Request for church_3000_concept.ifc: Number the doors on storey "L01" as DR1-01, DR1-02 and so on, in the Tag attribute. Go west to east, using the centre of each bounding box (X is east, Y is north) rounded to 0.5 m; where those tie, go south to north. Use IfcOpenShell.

First a look at what the model holds.

```python
import ifcopenshell
import ifcopenshell.util.element
import ifcopenshell.util.placement

model = ifcopenshell.open("church_3000_concept.ifc")
print(model.schema)
storey = next(s for s in model.by_type("IfcBuildingStorey") if s.Name == "L01")
doors = [e for e in ifcopenshell.util.element.get_decomposition(storey) if e.is_a("IfcDoor")]
for e in sorted(doors, key=lambda e: e.id()):
    origin = ifcopenshell.util.placement.get_local_placement(e.ObjectPlacement)[:3, 3]
    print(e.id(), e.Tag, e.Name, origin.round(2) + 0.0, sep=" | ")
```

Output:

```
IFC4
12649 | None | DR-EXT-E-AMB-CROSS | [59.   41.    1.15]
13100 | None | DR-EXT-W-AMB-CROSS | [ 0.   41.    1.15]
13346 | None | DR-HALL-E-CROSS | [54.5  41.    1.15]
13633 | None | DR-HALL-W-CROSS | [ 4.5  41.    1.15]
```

```python
import ifcopenshell
import ifcopenshell.geom
import ifcopenshell.util.element
import ifcopenshell.util.shape

model = ifcopenshell.open("church_3000_concept.ifc")
settings = ifcopenshell.geom.settings()
settings.set("use-world-coords", True)


def centre(element):
    shape = ifcopenshell.geom.create_shape(settings, element)
    return ifcopenshell.util.shape.get_bbox_centroid(shape.geometry)


storey = next(s for s in model.by_type("IfcBuildingStorey") if s.Name == "L01")
doors = [e for e in ifcopenshell.util.element.get_decomposition(storey) if e.is_a("IfcDoor")]

# Insertion points can sit at a corner or the storey origin, so sort by the geometry (in metres).
centres = {e: centre(e) for e in doors}
doors.sort(key=lambda e: (round(centres[e][0] / 0.5), centres[e][1]))

for i, e in enumerate(doors, start=1):
    number = f"DR1-{i:02d}"
    e.Tag = number
    print(e.id(), number)

model.write("church_3000_concept-out.ifc")
```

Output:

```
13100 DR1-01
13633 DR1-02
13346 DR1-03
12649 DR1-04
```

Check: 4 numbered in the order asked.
